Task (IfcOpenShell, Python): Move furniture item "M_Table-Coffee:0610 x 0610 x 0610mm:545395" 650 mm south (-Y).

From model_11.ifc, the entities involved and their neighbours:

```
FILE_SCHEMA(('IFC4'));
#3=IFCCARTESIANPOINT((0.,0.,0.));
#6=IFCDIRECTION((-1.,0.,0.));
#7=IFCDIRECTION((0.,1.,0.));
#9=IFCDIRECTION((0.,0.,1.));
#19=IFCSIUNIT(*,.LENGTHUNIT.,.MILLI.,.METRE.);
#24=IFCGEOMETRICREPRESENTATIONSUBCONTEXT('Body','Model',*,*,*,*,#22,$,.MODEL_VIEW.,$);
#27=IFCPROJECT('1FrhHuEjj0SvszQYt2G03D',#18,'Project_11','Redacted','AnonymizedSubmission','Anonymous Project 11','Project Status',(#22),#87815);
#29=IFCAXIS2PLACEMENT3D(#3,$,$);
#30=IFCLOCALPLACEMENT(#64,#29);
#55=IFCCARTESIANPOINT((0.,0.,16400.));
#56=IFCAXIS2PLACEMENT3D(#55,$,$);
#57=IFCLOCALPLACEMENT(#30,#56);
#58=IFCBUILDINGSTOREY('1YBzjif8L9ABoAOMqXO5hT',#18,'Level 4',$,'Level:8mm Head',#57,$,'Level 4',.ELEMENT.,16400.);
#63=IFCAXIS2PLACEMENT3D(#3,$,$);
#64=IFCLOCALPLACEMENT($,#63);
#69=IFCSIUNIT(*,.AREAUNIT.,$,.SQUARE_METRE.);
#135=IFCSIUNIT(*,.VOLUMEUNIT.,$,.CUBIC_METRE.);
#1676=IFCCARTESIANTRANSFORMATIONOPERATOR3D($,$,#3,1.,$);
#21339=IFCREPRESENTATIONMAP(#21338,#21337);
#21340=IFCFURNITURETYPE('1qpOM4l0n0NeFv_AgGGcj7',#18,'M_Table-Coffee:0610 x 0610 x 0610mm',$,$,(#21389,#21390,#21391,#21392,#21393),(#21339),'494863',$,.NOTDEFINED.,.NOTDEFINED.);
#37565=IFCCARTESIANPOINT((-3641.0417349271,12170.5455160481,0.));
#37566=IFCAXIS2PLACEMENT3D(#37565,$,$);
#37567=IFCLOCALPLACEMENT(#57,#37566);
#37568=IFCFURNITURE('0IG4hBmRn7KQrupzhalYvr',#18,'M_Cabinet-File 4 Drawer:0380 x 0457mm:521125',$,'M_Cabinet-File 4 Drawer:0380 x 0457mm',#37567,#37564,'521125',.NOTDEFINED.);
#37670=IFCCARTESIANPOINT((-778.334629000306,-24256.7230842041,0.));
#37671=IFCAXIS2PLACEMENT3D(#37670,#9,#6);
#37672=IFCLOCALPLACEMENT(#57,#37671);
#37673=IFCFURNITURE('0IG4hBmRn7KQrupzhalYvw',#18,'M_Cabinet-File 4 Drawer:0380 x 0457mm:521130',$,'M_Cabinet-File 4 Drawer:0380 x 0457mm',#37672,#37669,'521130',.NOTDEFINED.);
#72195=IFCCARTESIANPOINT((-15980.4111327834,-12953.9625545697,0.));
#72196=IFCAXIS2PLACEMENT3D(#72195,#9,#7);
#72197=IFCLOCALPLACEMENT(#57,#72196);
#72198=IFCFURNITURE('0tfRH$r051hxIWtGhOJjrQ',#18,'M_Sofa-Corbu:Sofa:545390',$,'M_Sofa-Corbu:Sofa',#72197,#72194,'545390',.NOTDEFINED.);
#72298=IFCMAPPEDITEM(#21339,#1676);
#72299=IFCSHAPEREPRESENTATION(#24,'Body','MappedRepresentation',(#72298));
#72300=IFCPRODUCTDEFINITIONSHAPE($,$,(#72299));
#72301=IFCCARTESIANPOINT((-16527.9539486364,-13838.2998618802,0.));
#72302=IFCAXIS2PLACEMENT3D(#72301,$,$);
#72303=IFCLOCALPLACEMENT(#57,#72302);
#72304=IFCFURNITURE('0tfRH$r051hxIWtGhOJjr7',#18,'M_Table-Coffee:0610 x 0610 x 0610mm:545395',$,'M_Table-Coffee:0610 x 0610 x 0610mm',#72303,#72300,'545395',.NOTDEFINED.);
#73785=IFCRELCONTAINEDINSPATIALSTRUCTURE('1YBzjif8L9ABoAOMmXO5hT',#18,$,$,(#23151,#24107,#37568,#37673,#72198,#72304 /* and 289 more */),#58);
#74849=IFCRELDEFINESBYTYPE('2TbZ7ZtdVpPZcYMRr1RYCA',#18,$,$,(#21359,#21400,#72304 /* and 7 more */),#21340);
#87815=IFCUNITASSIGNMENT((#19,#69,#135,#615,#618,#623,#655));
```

```python
import ifcopenshell
import ifcopenshell.api.geometry
import ifcopenshell.util.placement
import ifcopenshell.util.unit

model = ifcopenshell.open("model_11.ifc")
unit_scale = ifcopenshell.util.unit.calculate_unit_scale(model)

item = model.by_guid("0tfRH$r051hxIWtGhOJjr7")
matrix = ifcopenshell.util.placement.get_local_placement(item.ObjectPlacement)
matrix[1, 3] -= 0.65 / unit_scale
ifcopenshell.api.geometry.edit_object_placement(model, product=item, matrix=matrix, is_si=False)

print(ifcopenshell.util.placement.get_local_placement(item.ObjectPlacement).round(3) + 0.0)

model.write("model_11_rev.ifc")
```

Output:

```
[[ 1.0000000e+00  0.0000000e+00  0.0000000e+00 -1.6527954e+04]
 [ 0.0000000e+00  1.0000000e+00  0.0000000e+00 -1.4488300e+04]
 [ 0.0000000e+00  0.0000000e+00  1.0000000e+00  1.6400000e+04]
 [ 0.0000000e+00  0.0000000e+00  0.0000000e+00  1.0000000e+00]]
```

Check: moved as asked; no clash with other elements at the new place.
